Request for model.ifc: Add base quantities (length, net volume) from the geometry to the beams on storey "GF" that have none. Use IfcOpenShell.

First a look at what the model holds.

```python
import ifcopenshell
import ifcopenshell.util.element
import ifcopenshell.util.unit

model = ifcopenshell.open("model.ifc")
print(model.schema)
for unit_type in ("LENGTHUNIT", "AREAUNIT", "VOLUMEUNIT"):
    print(unit_type, ifcopenshell.util.unit.calculate_unit_scale(model, unit_type))
storey = next(s for s in model.by_type("IfcBuildingStorey") if s.Name == "GF")
beams = [e for e in ifcopenshell.util.element.get_decomposition(storey) if e.is_a("IfcBeam")]
for e in sorted(beams, key=lambda e: e.id()):
    print(e.id(), e.is_a(), e.Name, list(ifcopenshell.util.element.get_psets(e, qtos_only=True)), sep=" | ")
```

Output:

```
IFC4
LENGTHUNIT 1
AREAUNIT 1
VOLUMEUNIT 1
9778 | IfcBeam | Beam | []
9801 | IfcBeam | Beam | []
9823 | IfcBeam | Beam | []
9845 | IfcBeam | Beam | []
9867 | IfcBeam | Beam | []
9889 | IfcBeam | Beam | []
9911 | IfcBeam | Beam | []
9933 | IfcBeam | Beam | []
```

```python
import ifcopenshell
import ifcopenshell.api.pset
import ifcopenshell.geom
import ifcopenshell.util.element
import ifcopenshell.util.shape
import ifcopenshell.util.unit

model = ifcopenshell.open("model.ifc")
unit_scale = ifcopenshell.util.unit.calculate_unit_scale(model)
volume_scale = ifcopenshell.util.unit.calculate_unit_scale(model, "VOLUMEUNIT")
settings = ifcopenshell.geom.settings()

storey = next(s for s in model.by_type("IfcBuildingStorey") if s.Name == "GF")
beams = [e for e in ifcopenshell.util.element.get_decomposition(storey) if e.is_a("IfcBeam")]

for e in sorted(beams, key=lambda e: e.id()):
    if ifcopenshell.util.element.get_psets(e, qtos_only=True, should_inherit=False):
        continue
    # Geometry comes back in metres, in the element's own axes.
    shape = ifcopenshell.geom.create_shape(settings, e)
    values = {
        "Length": ifcopenshell.util.shape.get_max_xyz(shape.geometry) / unit_scale,
        "NetVolume": ifcopenshell.util.shape.get_volume(shape.geometry) / volume_scale,
    }
    qto = ifcopenshell.api.pset.add_qto(model, product=e, name="Qto_BeamBaseQuantities")
    ifcopenshell.api.pset.edit_qto(model, qto=qto, properties=values)
    print(e.id(), {k: round(v, 3) for k, v in values.items()})

model.write("model_edited.ifc")
```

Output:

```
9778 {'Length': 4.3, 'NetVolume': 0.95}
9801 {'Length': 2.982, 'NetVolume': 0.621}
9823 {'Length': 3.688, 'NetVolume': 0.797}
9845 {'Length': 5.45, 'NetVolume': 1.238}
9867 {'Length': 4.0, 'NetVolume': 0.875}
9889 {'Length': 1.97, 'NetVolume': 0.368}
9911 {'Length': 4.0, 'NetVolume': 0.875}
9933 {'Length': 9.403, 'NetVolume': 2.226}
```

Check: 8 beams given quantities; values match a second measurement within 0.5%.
